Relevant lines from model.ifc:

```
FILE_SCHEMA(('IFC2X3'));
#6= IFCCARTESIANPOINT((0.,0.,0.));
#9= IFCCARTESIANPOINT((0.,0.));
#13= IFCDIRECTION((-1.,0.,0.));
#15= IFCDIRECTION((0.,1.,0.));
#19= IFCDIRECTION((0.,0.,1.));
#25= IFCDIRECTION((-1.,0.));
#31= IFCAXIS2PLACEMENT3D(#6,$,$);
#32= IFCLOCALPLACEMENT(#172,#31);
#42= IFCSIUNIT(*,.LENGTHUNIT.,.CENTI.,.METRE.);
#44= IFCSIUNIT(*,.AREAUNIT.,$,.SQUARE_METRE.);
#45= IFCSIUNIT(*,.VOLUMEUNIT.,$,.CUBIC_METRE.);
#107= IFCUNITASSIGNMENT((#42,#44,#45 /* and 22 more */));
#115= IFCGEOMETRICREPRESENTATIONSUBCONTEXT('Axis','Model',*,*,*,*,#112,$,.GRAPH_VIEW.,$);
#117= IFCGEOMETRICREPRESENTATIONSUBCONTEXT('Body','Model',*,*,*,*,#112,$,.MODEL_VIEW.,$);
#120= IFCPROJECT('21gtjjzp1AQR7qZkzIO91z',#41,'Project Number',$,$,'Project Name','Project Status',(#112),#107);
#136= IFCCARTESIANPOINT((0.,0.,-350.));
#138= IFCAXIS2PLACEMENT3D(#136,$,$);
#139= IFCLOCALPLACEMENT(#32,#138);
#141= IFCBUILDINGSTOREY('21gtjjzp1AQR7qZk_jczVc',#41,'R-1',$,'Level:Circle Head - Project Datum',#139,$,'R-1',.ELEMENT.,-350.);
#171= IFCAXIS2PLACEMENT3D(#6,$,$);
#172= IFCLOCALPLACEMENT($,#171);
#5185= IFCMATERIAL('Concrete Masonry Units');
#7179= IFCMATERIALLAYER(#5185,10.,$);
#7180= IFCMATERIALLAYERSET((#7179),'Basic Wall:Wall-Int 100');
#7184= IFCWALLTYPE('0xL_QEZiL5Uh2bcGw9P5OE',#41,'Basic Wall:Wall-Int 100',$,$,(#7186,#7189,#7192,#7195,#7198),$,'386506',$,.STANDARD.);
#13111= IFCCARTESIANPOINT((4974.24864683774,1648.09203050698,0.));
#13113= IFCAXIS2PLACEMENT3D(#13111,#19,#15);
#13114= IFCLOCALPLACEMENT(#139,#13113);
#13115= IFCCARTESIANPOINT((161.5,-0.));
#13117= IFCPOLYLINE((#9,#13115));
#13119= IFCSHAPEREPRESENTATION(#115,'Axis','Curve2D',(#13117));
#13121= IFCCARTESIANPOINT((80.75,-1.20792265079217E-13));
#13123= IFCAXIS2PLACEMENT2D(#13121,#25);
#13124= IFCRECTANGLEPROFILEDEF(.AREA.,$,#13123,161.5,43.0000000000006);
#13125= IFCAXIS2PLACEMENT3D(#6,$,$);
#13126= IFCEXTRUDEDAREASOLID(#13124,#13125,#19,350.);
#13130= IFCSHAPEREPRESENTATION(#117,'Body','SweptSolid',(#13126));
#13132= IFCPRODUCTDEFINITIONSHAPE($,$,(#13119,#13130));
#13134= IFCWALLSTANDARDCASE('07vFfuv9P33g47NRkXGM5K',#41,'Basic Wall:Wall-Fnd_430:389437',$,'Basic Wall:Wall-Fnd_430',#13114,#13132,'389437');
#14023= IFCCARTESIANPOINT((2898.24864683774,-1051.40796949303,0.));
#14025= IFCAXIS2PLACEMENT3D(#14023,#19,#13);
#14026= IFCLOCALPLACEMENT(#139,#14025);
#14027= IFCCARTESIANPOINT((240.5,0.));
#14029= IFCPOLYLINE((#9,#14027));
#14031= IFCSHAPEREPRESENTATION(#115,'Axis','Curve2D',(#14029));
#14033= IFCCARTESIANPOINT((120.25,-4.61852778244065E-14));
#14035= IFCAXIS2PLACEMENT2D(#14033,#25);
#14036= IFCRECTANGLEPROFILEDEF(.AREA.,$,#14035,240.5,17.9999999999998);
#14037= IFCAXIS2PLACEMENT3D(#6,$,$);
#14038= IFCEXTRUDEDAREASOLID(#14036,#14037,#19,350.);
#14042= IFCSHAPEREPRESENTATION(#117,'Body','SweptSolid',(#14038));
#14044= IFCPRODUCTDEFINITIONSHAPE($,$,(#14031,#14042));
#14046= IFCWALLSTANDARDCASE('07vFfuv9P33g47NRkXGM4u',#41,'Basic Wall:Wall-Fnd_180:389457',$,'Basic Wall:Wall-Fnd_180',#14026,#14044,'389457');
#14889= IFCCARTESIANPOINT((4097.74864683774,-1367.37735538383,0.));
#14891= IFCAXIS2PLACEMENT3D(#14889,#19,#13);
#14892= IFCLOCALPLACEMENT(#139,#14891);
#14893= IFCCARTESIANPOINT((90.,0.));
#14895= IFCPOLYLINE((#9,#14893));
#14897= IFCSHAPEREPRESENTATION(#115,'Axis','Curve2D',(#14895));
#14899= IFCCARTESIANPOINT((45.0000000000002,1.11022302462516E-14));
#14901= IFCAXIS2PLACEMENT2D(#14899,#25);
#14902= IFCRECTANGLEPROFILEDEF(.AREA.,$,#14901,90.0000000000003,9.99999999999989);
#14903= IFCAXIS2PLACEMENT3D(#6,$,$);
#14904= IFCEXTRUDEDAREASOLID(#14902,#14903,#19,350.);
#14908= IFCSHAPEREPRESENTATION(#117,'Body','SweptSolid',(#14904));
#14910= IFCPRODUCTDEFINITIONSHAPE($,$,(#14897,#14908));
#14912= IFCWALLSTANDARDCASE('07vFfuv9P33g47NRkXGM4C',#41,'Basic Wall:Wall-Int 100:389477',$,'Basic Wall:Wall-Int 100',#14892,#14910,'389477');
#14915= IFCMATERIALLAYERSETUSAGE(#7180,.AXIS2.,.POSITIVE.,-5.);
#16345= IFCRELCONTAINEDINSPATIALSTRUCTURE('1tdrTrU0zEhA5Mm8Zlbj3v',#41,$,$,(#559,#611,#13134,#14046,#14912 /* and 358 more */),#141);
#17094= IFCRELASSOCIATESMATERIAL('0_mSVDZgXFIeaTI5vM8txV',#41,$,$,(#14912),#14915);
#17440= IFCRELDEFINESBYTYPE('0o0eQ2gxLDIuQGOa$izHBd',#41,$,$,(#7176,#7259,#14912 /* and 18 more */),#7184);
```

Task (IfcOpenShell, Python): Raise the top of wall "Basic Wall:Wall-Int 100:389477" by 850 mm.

```python
import ifcopenshell
import ifcopenshell.geom
import ifcopenshell.util.representation
import ifcopenshell.util.shape
import ifcopenshell.util.unit

model = ifcopenshell.open("model.ifc")
unit_scale = ifcopenshell.util.unit.calculate_unit_scale(model)
settings = ifcopenshell.geom.settings()


def volume(element):
    """Net volume in cubic metres, openings subtracted."""
    shape = ifcopenshell.geom.create_shape(settings, element)
    return ifcopenshell.util.shape.get_volume(shape.geometry)


wall = model.by_guid("07vFfuv9P33g47NRkXGM4C")
before = volume(wall)

body = ifcopenshell.util.representation.get_representation(wall, "Model", "Body")
solid = body.Items[0]
old_height = solid.Depth
solid.Depth += 0.85 / unit_scale
after = volume(wall)

print(f"height {old_height:g} -> {solid.Depth:g}, volume {before:.3f} -> {after:.3f} m3")

model.write("model_edited.ifc")
```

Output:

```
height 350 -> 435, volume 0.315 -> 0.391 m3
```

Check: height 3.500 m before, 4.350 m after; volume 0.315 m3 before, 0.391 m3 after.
